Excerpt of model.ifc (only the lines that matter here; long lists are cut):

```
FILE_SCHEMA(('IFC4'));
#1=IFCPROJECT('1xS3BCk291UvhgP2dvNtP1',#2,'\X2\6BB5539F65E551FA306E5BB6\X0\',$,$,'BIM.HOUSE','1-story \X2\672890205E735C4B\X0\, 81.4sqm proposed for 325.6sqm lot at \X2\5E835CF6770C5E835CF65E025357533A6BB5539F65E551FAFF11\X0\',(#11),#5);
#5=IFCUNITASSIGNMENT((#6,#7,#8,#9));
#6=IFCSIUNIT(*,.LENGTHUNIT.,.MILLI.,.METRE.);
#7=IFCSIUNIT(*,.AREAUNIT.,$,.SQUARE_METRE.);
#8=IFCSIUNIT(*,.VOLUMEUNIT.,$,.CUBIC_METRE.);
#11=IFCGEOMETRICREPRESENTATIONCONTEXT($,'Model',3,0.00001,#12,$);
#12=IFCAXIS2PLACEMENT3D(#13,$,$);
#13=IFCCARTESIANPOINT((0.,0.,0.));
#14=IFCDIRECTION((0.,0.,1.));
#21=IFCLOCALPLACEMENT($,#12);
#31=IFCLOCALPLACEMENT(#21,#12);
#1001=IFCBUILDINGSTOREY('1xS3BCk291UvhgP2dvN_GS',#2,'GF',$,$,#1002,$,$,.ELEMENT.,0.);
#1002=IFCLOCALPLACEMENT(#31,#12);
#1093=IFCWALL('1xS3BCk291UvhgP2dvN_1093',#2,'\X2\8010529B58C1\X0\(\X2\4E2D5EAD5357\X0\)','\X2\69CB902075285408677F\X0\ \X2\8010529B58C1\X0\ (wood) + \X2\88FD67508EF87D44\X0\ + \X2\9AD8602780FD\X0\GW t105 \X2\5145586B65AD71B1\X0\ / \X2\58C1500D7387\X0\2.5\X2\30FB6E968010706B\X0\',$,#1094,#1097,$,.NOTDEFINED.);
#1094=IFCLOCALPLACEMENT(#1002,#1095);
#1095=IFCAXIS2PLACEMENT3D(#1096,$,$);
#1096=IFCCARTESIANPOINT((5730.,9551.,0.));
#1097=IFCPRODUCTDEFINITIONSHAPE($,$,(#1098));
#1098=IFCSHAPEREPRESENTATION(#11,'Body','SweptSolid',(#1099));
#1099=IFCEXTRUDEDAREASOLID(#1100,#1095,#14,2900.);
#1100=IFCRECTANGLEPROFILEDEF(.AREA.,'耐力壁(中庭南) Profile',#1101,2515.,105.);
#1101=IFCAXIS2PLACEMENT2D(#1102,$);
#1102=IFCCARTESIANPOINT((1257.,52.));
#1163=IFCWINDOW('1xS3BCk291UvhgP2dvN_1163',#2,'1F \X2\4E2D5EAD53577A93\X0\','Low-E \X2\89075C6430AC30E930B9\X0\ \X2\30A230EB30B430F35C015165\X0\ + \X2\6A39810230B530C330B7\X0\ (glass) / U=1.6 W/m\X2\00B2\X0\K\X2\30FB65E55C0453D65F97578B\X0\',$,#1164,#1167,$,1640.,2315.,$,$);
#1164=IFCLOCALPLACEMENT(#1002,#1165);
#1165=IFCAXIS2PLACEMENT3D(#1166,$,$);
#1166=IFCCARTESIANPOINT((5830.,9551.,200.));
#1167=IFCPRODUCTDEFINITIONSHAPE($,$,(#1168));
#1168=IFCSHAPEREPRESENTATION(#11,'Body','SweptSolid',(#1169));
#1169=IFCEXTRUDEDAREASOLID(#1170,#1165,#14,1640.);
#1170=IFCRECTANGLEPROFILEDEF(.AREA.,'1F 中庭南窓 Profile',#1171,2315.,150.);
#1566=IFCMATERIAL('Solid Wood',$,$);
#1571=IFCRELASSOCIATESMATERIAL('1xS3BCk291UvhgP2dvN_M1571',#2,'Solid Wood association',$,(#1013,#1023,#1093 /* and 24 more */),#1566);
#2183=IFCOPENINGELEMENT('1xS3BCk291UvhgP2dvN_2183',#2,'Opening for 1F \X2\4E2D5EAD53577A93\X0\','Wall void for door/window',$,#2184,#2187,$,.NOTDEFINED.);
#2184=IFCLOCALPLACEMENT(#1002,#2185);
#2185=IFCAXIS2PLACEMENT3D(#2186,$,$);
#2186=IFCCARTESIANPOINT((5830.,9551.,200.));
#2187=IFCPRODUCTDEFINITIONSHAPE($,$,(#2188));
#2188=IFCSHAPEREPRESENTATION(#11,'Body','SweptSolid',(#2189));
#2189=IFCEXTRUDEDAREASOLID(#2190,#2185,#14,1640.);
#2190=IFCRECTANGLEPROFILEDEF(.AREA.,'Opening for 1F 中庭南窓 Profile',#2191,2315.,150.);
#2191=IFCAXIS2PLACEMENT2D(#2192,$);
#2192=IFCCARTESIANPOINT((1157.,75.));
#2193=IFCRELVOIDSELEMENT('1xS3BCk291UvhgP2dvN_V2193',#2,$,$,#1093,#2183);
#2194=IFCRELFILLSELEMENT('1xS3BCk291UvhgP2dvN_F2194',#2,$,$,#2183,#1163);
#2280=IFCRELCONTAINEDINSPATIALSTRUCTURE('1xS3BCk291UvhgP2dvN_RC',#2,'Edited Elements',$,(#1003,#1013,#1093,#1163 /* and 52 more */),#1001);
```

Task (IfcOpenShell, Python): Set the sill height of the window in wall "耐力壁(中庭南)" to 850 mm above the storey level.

```python
import numpy as np
import ifcopenshell
import ifcopenshell.api.geometry
import ifcopenshell.geom
import ifcopenshell.util.element
import ifcopenshell.util.placement
import ifcopenshell.util.shape
import ifcopenshell.util.unit

model = ifcopenshell.open("model.ifc")
unit_scale = ifcopenshell.util.unit.calculate_unit_scale(model)

window = model.by_id(1163)
opening = window.FillsVoids[0].RelatingOpeningElement
storey = ifcopenshell.util.element.get_container(window, ifc_class="IfcBuildingStorey")
level = ifcopenshell.util.placement.get_local_placement(storey.ObjectPlacement)[2, 3]

# The opening's origin need not be at the sill, so measure its lowest point.
shape = ifcopenshell.geom.create_shape(ifcopenshell.geom.settings(), opening)
bottom = ifcopenshell.util.shape.get_shape_bottom_elevation(shape, shape.geometry) / unit_scale
dz = level + 0.85 / unit_scale - bottom

shift = np.array([0.0, 0.0, dz])
# The window is not placed relative to its opening, so move both.
for product in (opening, window):
    matrix = ifcopenshell.util.placement.get_local_placement(product.ObjectPlacement)
    matrix[:3, 3] += shift
    ifcopenshell.api.geometry.edit_object_placement(model, product=product, matrix=matrix, is_si=False)

print(f"moved by {dz * unit_scale:+.3f} m")

model.write("model_v2.ifc")
```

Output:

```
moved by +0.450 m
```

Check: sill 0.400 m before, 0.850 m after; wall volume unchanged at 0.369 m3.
